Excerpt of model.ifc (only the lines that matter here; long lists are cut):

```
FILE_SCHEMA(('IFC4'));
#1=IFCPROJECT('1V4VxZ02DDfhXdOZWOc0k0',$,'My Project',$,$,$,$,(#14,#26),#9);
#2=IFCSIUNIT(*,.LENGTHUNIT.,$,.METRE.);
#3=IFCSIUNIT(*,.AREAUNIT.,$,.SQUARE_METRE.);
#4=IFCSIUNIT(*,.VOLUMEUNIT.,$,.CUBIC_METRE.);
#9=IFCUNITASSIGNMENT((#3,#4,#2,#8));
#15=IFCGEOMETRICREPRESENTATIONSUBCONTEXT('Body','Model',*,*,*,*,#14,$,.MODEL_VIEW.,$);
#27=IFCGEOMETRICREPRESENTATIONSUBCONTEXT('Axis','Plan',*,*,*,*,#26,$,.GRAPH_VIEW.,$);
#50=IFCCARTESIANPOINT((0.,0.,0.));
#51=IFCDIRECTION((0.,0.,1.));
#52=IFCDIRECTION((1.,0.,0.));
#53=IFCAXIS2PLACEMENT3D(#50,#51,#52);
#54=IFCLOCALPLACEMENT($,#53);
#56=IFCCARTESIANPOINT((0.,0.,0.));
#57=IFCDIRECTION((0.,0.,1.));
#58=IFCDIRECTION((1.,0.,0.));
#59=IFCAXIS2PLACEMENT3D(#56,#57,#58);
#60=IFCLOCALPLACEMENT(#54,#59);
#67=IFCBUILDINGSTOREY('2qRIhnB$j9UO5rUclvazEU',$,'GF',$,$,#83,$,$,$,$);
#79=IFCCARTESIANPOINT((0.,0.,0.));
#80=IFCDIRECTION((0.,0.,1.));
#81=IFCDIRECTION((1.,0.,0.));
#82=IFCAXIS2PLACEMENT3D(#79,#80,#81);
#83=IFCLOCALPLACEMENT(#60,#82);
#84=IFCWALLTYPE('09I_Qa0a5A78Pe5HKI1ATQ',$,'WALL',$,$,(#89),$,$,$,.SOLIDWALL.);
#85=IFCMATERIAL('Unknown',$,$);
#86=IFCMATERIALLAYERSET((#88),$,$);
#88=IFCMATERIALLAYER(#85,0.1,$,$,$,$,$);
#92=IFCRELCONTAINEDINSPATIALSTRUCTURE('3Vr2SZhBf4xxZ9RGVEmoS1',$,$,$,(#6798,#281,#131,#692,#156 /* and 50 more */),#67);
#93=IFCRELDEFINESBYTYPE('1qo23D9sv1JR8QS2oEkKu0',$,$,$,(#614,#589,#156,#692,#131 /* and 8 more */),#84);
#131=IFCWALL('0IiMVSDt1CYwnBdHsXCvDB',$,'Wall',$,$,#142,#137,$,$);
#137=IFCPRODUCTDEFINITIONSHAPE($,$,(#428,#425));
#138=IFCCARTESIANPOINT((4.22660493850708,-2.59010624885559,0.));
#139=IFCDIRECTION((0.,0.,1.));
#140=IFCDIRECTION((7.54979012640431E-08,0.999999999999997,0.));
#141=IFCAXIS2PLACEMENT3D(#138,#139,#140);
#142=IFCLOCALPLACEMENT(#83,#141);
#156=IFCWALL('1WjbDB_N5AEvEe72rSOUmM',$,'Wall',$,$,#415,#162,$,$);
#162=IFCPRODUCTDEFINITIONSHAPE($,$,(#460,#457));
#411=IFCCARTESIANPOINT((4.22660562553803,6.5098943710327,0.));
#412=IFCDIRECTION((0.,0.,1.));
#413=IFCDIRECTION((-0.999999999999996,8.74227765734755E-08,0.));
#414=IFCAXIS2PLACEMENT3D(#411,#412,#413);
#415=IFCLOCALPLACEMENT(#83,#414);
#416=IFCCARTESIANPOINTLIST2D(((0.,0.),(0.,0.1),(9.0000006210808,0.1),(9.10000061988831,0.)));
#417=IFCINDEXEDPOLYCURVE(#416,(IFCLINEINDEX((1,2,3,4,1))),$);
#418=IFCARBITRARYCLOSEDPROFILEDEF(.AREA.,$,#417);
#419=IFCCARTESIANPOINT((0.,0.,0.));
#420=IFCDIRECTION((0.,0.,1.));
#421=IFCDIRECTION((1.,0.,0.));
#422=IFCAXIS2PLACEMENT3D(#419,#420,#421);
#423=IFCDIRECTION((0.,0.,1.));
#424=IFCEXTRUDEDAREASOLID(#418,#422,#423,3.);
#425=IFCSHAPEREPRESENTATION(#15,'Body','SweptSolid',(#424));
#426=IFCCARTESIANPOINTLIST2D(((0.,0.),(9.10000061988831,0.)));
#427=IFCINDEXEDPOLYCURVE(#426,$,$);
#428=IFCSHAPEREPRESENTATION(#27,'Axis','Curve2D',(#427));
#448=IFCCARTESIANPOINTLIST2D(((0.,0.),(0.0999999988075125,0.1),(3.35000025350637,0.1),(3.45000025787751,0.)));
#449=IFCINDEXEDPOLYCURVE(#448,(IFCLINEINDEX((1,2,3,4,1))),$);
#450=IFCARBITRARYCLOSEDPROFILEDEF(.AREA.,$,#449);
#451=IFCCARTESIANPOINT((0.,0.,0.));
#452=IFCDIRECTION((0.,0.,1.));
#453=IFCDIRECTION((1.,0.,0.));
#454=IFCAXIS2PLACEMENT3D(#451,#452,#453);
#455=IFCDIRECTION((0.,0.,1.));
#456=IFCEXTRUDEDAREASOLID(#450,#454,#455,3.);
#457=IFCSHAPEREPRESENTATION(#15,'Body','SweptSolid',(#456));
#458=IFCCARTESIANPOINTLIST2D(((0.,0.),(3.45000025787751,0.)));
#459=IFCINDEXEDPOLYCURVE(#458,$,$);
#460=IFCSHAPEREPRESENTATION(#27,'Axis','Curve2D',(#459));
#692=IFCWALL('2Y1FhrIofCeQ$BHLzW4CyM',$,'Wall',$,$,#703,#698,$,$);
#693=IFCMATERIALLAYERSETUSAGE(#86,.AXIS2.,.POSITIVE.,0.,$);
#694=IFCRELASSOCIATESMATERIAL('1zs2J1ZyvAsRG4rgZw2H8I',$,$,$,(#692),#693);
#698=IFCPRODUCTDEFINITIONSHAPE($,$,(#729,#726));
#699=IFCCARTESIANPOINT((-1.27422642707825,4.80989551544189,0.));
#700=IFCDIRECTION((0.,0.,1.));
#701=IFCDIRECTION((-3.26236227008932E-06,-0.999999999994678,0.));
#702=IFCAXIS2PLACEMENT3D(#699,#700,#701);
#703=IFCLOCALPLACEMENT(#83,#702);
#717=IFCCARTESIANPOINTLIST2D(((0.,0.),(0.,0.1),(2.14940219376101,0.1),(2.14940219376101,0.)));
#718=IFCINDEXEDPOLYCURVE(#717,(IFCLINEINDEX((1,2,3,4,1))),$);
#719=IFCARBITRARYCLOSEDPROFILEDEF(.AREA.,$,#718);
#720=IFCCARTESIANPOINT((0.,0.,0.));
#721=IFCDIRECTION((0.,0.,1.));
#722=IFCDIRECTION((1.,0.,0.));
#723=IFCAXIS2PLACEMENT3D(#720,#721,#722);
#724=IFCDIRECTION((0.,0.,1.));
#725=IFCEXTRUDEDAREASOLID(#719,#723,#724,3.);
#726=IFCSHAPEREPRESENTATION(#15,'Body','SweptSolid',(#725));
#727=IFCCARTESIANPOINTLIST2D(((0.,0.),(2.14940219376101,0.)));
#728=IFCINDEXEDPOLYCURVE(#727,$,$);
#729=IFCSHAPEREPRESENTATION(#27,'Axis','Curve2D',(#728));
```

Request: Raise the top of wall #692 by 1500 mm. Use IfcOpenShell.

```python
import ifcopenshell
import ifcopenshell.geom
import ifcopenshell.util.representation
import ifcopenshell.util.shape

model = ifcopenshell.open("model.ifc")
settings = ifcopenshell.geom.settings()


def volume(element):
    """Net volume in cubic metres, openings subtracted."""
    shape = ifcopenshell.geom.create_shape(settings, element)
    return ifcopenshell.util.shape.get_volume(shape.geometry)


wall = model.by_id(692)
before = volume(wall)

body = ifcopenshell.util.representation.get_representation(wall, "Model", "Body")
solid = body.Items[0]
old_height = solid.Depth
solid.Depth += 1.5
after = volume(wall)

print(f"height {old_height:g} -> {solid.Depth:g}, volume {before:.3f} -> {after:.3f} m3")

model.write("model_edited.ifc")
```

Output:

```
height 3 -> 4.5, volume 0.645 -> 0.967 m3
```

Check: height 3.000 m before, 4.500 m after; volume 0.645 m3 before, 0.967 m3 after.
